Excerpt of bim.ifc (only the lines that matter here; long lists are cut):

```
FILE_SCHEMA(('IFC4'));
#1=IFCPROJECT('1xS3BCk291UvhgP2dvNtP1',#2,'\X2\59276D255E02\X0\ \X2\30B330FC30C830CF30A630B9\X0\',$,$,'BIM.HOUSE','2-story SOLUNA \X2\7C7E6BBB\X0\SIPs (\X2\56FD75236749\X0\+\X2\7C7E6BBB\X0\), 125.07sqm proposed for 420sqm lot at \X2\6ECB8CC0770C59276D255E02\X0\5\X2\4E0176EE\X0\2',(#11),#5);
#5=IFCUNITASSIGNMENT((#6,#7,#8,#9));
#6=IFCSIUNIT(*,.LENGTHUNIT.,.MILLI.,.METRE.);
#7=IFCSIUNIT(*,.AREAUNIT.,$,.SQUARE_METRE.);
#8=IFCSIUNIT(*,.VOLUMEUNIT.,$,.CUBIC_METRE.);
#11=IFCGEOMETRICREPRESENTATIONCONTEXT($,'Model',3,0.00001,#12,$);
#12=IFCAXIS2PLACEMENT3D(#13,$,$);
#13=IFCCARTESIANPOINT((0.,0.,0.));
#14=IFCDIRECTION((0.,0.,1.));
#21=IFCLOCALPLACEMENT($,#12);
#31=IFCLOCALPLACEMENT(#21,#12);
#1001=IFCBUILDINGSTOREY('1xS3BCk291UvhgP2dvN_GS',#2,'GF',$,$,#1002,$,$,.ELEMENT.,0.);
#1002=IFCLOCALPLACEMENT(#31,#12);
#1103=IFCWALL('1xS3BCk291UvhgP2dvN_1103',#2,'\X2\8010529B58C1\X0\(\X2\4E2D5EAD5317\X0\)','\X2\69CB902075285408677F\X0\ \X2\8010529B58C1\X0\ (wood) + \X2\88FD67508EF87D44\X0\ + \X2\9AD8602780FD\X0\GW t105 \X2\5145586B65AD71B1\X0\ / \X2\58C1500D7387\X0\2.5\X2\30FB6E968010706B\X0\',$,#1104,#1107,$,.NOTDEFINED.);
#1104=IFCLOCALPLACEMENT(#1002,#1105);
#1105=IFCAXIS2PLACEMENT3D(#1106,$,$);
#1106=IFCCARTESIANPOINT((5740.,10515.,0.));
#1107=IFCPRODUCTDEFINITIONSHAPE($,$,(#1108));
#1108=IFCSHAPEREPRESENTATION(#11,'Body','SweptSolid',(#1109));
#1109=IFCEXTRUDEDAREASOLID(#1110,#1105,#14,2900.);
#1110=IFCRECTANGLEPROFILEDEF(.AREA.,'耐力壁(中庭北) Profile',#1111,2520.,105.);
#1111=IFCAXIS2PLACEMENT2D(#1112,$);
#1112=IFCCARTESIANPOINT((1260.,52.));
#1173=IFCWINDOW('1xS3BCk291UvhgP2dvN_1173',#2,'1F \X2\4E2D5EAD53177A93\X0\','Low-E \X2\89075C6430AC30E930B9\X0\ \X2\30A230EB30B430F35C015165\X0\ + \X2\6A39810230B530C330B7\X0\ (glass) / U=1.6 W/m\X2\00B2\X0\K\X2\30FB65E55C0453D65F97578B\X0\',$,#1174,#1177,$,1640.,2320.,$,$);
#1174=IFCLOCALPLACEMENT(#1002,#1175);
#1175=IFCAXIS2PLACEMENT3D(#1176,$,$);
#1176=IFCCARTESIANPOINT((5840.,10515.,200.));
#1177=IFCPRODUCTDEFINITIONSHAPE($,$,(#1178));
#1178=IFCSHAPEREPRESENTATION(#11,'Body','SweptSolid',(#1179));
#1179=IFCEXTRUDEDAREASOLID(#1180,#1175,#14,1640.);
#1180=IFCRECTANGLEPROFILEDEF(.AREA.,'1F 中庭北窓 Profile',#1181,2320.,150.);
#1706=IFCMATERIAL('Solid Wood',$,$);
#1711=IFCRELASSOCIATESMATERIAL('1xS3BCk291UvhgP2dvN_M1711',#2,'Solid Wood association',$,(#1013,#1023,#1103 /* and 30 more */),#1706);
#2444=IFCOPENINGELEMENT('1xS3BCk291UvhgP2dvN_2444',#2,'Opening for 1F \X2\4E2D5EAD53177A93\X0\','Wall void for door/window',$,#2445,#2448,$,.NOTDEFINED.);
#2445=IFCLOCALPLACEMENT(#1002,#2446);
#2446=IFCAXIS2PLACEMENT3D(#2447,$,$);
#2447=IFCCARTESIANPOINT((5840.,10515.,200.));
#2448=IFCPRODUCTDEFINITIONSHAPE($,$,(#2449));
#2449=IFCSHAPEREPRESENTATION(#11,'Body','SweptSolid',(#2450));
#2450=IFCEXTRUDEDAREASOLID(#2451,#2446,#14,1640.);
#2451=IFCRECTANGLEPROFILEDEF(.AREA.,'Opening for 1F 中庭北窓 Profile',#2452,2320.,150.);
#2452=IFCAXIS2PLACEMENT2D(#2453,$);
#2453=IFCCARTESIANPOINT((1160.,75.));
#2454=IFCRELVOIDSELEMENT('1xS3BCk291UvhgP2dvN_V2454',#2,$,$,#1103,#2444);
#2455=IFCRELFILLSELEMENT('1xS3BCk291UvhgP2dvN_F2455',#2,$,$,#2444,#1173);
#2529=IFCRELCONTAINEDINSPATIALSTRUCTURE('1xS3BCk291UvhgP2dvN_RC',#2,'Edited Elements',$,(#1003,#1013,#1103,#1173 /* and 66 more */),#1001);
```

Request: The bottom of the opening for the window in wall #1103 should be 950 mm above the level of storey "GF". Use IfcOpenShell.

```python
import numpy as np
import ifcopenshell
import ifcopenshell.api.geometry
import ifcopenshell.geom
import ifcopenshell.util.element
import ifcopenshell.util.placement
import ifcopenshell.util.shape
import ifcopenshell.util.unit

model = ifcopenshell.open("bim.ifc")
unit_scale = ifcopenshell.util.unit.calculate_unit_scale(model)

window = model.by_id(1173)
opening = window.FillsVoids[0].RelatingOpeningElement
storey = ifcopenshell.util.element.get_container(window, ifc_class="IfcBuildingStorey")
level = ifcopenshell.util.placement.get_local_placement(storey.ObjectPlacement)[2, 3]

# The opening's origin need not be at the sill, so measure its lowest point.
shape = ifcopenshell.geom.create_shape(ifcopenshell.geom.settings(), opening)
bottom = ifcopenshell.util.shape.get_shape_bottom_elevation(shape, shape.geometry) / unit_scale
dz = level + 0.95 / unit_scale - bottom

shift = np.array([0.0, 0.0, dz])
# The window is not placed relative to its opening, so move both.
for product in (opening, window):
    matrix = ifcopenshell.util.placement.get_local_placement(product.ObjectPlacement)
    matrix[:3, 3] += shift
    ifcopenshell.api.geometry.edit_object_placement(model, product=product, matrix=matrix, is_si=False)

print(f"moved by {dz * unit_scale:+.3f} m")

model.write("bim_updated.ifc")
```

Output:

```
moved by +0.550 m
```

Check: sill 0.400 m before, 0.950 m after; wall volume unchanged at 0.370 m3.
